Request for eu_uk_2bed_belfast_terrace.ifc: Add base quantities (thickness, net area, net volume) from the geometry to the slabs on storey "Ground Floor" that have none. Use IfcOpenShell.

First a look at what the model holds.

```python
import ifcopenshell
import ifcopenshell.util.element
import ifcopenshell.util.unit

model = ifcopenshell.open("eu_uk_2bed_belfast_terrace.ifc")
print(model.schema)
for unit_type in ("LENGTHUNIT", "AREAUNIT", "VOLUMEUNIT"):
    print(unit_type, ifcopenshell.util.unit.calculate_unit_scale(model, unit_type))
storey = next(s for s in model.by_type("IfcBuildingStorey") if s.Name == "Ground Floor")
slabs = [e for e in ifcopenshell.util.element.get_decomposition(storey) if e.is_a("IfcSlab")]
for e in sorted(slabs, key=lambda e: e.id()):
    print(e.id(), e.is_a(), e.Name, list(ifcopenshell.util.element.get_psets(e, qtos_only=True)), sep=" | ")
```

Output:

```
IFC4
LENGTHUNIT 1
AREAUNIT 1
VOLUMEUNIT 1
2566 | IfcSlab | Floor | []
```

```python
import ifcopenshell
import ifcopenshell.api.pset
import ifcopenshell.geom
import ifcopenshell.util.element
import ifcopenshell.util.shape
import ifcopenshell.util.unit

model = ifcopenshell.open("eu_uk_2bed_belfast_terrace.ifc")
unit_scale = ifcopenshell.util.unit.calculate_unit_scale(model)
area_scale = ifcopenshell.util.unit.calculate_unit_scale(model, "AREAUNIT")
volume_scale = ifcopenshell.util.unit.calculate_unit_scale(model, "VOLUMEUNIT")
settings = ifcopenshell.geom.settings()

storey = next(s for s in model.by_type("IfcBuildingStorey") if s.Name == "Ground Floor")
slabs = [e for e in ifcopenshell.util.element.get_decomposition(storey) if e.is_a("IfcSlab")]

for e in sorted(slabs, key=lambda e: e.id()):
    if ifcopenshell.util.element.get_psets(e, qtos_only=True, should_inherit=False):
        continue
    # Geometry comes back in metres, in the element's own axes.
    shape = ifcopenshell.geom.create_shape(settings, e)
    values = {
        "Width": ifcopenshell.util.shape.get_z(shape.geometry) / unit_scale,
        "NetArea": ifcopenshell.util.shape.get_footprint_area(shape.geometry) / area_scale,
        "NetVolume": ifcopenshell.util.shape.get_volume(shape.geometry) / volume_scale,
    }
    qto = ifcopenshell.api.pset.add_qto(model, product=e, name="Qto_SlabBaseQuantities")
    ifcopenshell.api.pset.edit_qto(model, qto=qto, properties=values)
    print(e.id(), {k: round(v, 3) for k, v in values.items()})

model.write("eu_uk_2bed_belfast_terrace_v2.ifc")
```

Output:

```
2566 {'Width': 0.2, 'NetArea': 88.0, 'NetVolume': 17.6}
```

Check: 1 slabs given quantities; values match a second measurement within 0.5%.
